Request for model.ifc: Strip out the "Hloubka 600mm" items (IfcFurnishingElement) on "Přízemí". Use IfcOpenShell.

First a look at what the model holds.

```python
import ifcopenshell
import ifcopenshell.util.element

model = ifcopenshell.open("model.ifc")
print(model.schema)
storey = next(s for s in model.by_type("IfcBuildingStorey") if s.Name == "Přízemí")
furniture = [e for e in ifcopenshell.util.element.get_decomposition(storey) if e.is_a("IfcFurnishingElement")]
seen = {}
for e in furniture:
    element_type = ifcopenshell.util.element.get_type(e)
    name = element_type.Name if element_type not in (None, e) else None
    seen[name] = seen.get(name, 0) + 1
for name, count in sorted(seen.items(), key=str):
    print(count, "x", name)
```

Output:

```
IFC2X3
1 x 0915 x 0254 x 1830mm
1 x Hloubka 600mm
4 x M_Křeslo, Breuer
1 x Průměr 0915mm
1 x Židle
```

```python
import ifcopenshell
import ifcopenshell.api.root
import ifcopenshell.util.element

model = ifcopenshell.open("model.ifc")

storey = next(s for s in model.by_type("IfcBuildingStorey") if s.Name == "Přízemí")
furniture = [e for e in ifcopenshell.util.element.get_decomposition(storey) if e.is_a("IfcFurnishingElement")]
targets = [e for e in furniture if (t := ifcopenshell.util.element.get_type(e)) not in (None, e) and t.Name == "Hloubka 600mm"]

for e in targets:
    ifcopenshell.api.root.remove_product(model, product=e)
print(len(targets), "removed")

model.write("model_rev.ifc")
```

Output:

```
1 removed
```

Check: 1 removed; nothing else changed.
